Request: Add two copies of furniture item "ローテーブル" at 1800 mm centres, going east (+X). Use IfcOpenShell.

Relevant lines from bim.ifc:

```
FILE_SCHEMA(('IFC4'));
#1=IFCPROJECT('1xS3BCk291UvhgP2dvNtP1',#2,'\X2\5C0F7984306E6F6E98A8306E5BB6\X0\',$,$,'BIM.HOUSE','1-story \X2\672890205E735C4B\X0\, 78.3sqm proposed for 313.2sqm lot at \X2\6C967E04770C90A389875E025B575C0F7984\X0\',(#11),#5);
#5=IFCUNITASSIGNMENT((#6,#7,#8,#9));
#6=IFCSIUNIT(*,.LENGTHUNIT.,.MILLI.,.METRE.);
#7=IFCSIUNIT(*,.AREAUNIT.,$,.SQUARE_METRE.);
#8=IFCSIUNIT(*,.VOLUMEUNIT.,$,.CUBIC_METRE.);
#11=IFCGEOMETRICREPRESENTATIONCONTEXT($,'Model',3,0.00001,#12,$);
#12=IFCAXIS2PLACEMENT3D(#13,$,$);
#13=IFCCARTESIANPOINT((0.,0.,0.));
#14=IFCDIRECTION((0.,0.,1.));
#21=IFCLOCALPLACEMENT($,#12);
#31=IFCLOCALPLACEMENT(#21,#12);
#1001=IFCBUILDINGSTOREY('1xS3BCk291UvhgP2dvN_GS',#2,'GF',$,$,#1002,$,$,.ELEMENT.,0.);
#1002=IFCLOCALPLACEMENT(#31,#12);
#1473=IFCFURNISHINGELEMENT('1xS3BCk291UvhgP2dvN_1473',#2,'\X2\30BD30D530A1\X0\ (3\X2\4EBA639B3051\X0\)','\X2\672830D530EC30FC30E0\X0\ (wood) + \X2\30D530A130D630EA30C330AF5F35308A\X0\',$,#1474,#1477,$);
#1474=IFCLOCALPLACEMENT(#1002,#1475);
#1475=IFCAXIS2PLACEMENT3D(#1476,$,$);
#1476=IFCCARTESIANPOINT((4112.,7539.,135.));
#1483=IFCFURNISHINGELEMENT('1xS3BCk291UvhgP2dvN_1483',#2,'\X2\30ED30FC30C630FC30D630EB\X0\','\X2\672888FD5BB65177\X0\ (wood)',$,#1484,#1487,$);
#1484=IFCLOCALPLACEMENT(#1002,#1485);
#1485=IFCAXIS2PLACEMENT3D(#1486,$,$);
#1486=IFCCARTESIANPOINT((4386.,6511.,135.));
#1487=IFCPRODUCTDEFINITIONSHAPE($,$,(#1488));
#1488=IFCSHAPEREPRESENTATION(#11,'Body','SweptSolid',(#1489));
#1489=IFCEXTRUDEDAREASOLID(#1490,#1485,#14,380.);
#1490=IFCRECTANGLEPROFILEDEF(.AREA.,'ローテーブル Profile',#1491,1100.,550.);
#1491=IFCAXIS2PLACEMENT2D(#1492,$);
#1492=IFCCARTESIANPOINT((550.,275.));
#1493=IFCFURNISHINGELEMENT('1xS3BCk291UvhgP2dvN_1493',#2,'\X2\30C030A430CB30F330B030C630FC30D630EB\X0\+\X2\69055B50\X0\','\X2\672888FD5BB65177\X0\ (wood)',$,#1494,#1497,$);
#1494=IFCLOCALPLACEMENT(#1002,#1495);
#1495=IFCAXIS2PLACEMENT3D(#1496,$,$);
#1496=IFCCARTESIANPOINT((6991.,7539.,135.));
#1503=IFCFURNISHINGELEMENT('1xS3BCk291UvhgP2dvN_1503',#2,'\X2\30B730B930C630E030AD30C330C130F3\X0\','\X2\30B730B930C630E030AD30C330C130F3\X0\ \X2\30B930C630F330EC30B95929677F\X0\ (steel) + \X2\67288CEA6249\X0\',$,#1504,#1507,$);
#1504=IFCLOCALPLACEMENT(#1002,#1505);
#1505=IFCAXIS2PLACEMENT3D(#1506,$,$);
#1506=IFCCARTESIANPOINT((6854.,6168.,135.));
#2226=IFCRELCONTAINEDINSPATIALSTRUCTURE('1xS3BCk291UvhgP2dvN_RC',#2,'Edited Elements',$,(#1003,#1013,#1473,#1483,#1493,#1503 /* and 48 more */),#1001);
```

```python
import numpy as np
import ifcopenshell
import ifcopenshell.api.geometry
import ifcopenshell.api.root
import ifcopenshell.util.element
import ifcopenshell.util.placement
import ifcopenshell.util.unit

model = ifcopenshell.open("bim.ifc")
unit_scale = ifcopenshell.util.unit.calculate_unit_scale(model)


def reuse_history(source, copy):
    """copy_class also copies each property set's owner history, people and application; keep the originals."""
    for rel in copy.IsDefinedBy:
        if rel.is_a("IfcRelDefinesByProperties") and (history := rel.RelatingPropertyDefinition.OwnerHistory):
            rel.RelatingPropertyDefinition.OwnerHistory = source.OwnerHistory
            ifcopenshell.util.element.remove_deep2(model, history)


source = model.by_guid("1xS3BCk291UvhgP2dvN_1483")
base = ifcopenshell.util.placement.get_local_placement(source.ObjectPlacement)
step = np.array([1.0, 0.0, 0.0]) * 1.8 / unit_scale

for i in range(1, 3):
    copy = ifcopenshell.api.root.copy_class(model, product=source)
    copy.Representation = ifcopenshell.util.element.copy_deep(
        model, source.Representation, exclude=["IfcGeometricRepresentationContext", "IfcRepresentationMap"]
    )
    reuse_history(source, copy)
    matrix = base.copy()
    matrix[:3, 3] += i * step
    print("added at", matrix[:3, 3].round(3) + 0.0)
    ifcopenshell.api.geometry.edit_object_placement(model, product=copy, matrix=matrix, is_si=False)

model.write("bim_edited.ifc")
```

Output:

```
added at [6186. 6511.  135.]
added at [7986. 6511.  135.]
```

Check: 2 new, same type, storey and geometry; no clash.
